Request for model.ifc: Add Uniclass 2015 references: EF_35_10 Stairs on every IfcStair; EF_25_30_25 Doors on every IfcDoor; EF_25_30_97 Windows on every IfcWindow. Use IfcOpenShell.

First a look at what the model holds.

```python
import ifcopenshell

model = ifcopenshell.open("model.ifc")
print(model.schema)
print("classifications:", [c.Name for c in model.by_type("IfcClassification")])
for ifc_class in ("IfcDoor", "IfcRoof", "IfcStair", "IfcWall", "IfcWindow"):
    print(ifc_class, len(model.by_type(ifc_class)))
```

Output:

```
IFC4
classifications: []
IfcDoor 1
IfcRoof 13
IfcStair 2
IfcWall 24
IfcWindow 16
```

```python
import ifcopenshell
import ifcopenshell.api.classification

model = ifcopenshell.open("model.ifc")

system = ifcopenshell.api.classification.add_classification(model, classification="Uniclass 2015")

codes = {
    "IfcStair": ("EF_35_10", "Stairs"),
    "IfcDoor": ("EF_25_30_25", "Doors"),
    "IfcWindow": ("EF_25_30_97", "Windows"),
}
for ifc_class, (code, name) in codes.items():
    products = model.by_type(ifc_class)
    ifcopenshell.api.classification.add_reference(
        model, products=products, classification=system, identification=code, name=name
    )
    print(code, len(products))

model.write("model-out.ifc")
```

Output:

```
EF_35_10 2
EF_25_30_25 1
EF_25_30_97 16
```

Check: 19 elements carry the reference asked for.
